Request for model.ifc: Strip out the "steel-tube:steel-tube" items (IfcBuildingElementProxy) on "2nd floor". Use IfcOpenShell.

First a look at what the model holds.

```python
import ifcopenshell
import ifcopenshell.util.element

model = ifcopenshell.open("model.ifc")
print(model.schema)
storey = next(s for s in model.by_type("IfcBuildingStorey") if s.Name == "2nd floor")
proxies = [e for e in ifcopenshell.util.element.get_decomposition(storey) if e.is_a("IfcBuildingElementProxy")]
seen = {}
for e in proxies:
    element_type = ifcopenshell.util.element.get_type(e)
    name = element_type.Name if element_type not in (None, e) else None
    seen[name] = seen.get(name, 0) + 1
for name, count in sorted(seen.items(), key=str):
    print(count, "x", name)
```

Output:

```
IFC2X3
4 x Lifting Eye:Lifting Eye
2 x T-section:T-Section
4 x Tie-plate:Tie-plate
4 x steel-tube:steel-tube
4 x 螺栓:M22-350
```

```python
import ifcopenshell
import ifcopenshell.api.root
import ifcopenshell.util.element

model = ifcopenshell.open("model.ifc")

storey = next(s for s in model.by_type("IfcBuildingStorey") if s.Name == "2nd floor")
proxies = [e for e in ifcopenshell.util.element.get_decomposition(storey) if e.is_a("IfcBuildingElementProxy")]
targets = [e for e in proxies if (t := ifcopenshell.util.element.get_type(e)) not in (None, e) and t.Name == "steel-tube:steel-tube"]

for e in targets:
    ifcopenshell.api.root.remove_product(model, product=e)
print(len(targets), "removed")

model.write("model-out.ifc")
```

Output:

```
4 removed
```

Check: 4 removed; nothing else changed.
